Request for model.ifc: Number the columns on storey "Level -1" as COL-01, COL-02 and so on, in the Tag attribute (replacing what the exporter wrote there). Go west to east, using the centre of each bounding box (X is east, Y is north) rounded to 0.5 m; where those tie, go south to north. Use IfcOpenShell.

First a look at what the model holds.

```python
import ifcopenshell
import ifcopenshell.util.element
import ifcopenshell.util.placement

model = ifcopenshell.open("model.ifc")
print(model.schema)
storey = next(s for s in model.by_type("IfcBuildingStorey") if s.Name == "Level -1")
columns = [e for e in ifcopenshell.util.element.get_decomposition(storey) if e.is_a("IfcColumn")]
for e in sorted(columns, key=lambda e: e.id()):
    origin = ifcopenshell.util.placement.get_local_placement(e.ObjectPlacement)[:3, 3]
    print(e.id(), e.Tag, e.Name, origin.round(2) + 0.0, sep=" | ")
```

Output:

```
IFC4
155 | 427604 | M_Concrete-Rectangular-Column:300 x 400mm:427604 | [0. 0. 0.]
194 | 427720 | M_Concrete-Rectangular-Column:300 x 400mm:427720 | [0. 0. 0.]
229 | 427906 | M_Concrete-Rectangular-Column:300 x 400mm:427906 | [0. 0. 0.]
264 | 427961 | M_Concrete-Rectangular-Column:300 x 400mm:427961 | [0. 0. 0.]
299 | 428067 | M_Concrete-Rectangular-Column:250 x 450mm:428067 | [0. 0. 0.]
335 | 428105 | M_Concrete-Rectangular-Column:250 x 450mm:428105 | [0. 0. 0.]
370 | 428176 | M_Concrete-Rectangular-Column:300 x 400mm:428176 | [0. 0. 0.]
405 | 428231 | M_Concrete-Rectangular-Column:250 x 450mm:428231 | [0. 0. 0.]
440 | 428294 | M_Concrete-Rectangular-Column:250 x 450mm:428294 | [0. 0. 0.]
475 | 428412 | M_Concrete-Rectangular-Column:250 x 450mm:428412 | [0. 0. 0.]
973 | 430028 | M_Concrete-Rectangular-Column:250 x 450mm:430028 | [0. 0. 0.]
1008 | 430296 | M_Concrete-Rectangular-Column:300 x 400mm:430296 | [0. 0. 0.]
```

```python
import ifcopenshell
import ifcopenshell.geom
import ifcopenshell.util.element
import ifcopenshell.util.shape

model = ifcopenshell.open("model.ifc")
settings = ifcopenshell.geom.settings()
settings.set("use-world-coords", True)


def centre(element):
    shape = ifcopenshell.geom.create_shape(settings, element)
    return ifcopenshell.util.shape.get_bbox_centroid(shape.geometry)


storey = next(s for s in model.by_type("IfcBuildingStorey") if s.Name == "Level -1")
columns = [e for e in ifcopenshell.util.element.get_decomposition(storey) if e.is_a("IfcColumn")]

# Insertion points can sit at a corner or the storey origin, so sort by the geometry (in metres).
centres = {e: centre(e) for e in columns}
columns.sort(key=lambda e: (round(centres[e][0] / 0.5), centres[e][1]))

for i, e in enumerate(columns, start=1):
    number = f"COL-{i:02d}"
    e.Tag = number
    print(e.id(), number)

model.write("model_edited.ifc")
```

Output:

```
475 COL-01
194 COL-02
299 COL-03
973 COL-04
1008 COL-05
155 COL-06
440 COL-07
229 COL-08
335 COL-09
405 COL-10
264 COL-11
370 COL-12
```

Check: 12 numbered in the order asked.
